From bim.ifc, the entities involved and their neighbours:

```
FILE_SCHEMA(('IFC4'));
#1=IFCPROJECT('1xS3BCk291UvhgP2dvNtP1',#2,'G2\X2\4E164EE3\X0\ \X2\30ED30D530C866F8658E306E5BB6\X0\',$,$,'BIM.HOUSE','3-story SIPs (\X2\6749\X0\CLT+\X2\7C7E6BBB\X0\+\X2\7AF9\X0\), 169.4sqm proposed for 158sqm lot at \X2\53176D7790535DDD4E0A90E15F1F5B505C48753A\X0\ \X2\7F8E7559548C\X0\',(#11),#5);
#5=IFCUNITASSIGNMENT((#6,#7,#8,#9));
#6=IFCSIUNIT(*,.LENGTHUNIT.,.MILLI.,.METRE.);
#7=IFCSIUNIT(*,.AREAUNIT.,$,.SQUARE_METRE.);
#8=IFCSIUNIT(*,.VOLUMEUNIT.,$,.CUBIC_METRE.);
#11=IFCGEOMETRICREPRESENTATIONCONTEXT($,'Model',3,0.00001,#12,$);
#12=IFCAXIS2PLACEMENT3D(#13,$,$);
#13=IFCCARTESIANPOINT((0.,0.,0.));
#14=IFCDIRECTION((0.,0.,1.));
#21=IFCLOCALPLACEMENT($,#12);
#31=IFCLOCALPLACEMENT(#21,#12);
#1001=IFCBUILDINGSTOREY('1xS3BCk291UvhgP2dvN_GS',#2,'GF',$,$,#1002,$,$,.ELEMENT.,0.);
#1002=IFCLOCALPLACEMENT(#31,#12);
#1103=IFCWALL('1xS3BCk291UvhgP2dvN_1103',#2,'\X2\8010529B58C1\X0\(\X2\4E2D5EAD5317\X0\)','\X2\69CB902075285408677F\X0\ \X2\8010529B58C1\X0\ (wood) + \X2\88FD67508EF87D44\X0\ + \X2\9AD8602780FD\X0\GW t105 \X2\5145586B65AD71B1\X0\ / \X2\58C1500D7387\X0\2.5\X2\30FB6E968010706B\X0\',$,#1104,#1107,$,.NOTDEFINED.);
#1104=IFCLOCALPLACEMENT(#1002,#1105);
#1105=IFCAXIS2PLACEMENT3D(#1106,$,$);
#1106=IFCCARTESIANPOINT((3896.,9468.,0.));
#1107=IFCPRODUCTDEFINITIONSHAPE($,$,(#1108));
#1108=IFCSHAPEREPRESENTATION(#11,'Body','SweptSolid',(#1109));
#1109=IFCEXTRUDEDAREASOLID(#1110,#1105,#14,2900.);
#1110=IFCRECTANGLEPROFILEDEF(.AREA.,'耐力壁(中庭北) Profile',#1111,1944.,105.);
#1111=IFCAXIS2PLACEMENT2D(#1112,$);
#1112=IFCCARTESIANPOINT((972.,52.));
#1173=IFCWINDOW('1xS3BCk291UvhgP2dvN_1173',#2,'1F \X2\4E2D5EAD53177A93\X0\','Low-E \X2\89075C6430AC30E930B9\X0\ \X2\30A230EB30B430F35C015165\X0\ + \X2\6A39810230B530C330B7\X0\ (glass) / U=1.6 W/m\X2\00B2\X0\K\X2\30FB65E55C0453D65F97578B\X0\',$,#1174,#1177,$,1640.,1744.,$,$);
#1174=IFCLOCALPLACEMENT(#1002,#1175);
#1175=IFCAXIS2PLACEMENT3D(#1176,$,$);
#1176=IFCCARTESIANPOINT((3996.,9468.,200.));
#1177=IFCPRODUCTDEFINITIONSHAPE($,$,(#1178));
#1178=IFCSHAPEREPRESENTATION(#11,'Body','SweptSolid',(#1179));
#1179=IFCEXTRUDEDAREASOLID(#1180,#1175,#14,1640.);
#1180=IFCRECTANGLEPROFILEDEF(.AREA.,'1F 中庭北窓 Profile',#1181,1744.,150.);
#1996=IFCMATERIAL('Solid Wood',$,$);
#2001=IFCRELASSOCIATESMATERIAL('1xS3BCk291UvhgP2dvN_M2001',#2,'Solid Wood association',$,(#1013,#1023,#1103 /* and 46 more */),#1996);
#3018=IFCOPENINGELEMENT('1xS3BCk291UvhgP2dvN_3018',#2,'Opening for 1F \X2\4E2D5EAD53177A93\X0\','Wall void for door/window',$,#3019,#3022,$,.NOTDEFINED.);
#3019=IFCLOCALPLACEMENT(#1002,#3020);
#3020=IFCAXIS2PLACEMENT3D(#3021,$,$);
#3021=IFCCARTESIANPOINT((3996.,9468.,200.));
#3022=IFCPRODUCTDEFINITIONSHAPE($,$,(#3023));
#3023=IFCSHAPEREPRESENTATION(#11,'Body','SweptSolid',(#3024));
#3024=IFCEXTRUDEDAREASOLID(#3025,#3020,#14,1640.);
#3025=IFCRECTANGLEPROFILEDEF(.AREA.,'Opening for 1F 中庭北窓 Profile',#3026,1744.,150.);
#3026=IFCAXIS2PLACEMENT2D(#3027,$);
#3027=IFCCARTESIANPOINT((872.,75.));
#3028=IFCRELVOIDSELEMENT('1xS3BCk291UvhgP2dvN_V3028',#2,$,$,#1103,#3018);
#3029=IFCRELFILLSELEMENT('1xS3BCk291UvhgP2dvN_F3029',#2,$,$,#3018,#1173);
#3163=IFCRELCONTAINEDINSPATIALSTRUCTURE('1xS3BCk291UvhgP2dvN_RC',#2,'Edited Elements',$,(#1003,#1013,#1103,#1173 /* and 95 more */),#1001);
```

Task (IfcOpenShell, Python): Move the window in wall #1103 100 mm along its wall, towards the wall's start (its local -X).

```python
import ifcopenshell
import ifcopenshell.api.geometry
import ifcopenshell.util.placement
import ifcopenshell.util.unit

model = ifcopenshell.open("bim.ifc")
unit_scale = ifcopenshell.util.unit.calculate_unit_scale(model)

window = model.by_guid("1xS3BCk291UvhgP2dvN_1173")
opening = window.FillsVoids[0].RelatingOpeningElement
wall = opening.VoidsElements[0].RelatingBuildingElement

wall_matrix = ifcopenshell.util.placement.get_local_placement(wall.ObjectPlacement)
shift = wall_matrix[:3, 0] * -0.1 / unit_scale
before = ifcopenshell.util.placement.get_local_placement(window.ObjectPlacement)[:3, 3].copy()

# The window is not placed relative to its opening, so move both.
for product in (opening, window):
    matrix = ifcopenshell.util.placement.get_local_placement(product.ObjectPlacement)
    matrix[:3, 3] += shift
    ifcopenshell.api.geometry.edit_object_placement(model, product=product, matrix=matrix, is_si=False)

after = ifcopenshell.util.placement.get_local_placement(window.ObjectPlacement)[:3, 3]
print("window moved by", (after - before).round(3) + 0.0)

model.write("bim_rev.ifc")
```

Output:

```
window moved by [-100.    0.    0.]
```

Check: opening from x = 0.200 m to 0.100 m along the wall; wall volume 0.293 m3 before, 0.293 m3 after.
